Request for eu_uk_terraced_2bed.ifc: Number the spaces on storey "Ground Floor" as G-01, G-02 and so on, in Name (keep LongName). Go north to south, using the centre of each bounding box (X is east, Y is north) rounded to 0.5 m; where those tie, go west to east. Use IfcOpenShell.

First a look at what the model holds.

```python
import ifcopenshell
import ifcopenshell.util.element
import ifcopenshell.util.placement

model = ifcopenshell.open("eu_uk_terraced_2bed.ifc")
print(model.schema)
storey = next(s for s in model.by_type("IfcBuildingStorey") if s.Name == "Ground Floor")
spaces = [e for e in ifcopenshell.util.element.get_decomposition(storey) if e.is_a("IfcSpace")]
for e in sorted(spaces, key=lambda e: e.id()):
    origin = ifcopenshell.util.placement.get_local_placement(e.ObjectPlacement)[:3, 3]
    print(e.id(), e.Name, e.LongName, origin.round(2) + 0.0, sep=" | ")
```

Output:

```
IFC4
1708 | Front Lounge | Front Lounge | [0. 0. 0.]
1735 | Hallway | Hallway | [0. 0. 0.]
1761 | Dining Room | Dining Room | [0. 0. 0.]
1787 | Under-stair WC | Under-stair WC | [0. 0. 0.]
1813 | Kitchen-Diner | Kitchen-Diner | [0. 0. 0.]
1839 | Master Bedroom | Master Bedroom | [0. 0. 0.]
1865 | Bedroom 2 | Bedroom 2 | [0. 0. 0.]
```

```python
import ifcopenshell
import ifcopenshell.geom
import ifcopenshell.util.element
import ifcopenshell.util.shape

model = ifcopenshell.open("eu_uk_terraced_2bed.ifc")
settings = ifcopenshell.geom.settings()
settings.set("use-world-coords", True)


def centre(element):
    shape = ifcopenshell.geom.create_shape(settings, element)
    return ifcopenshell.util.shape.get_bbox_centroid(shape.geometry)


storey = next(s for s in model.by_type("IfcBuildingStorey") if s.Name == "Ground Floor")
spaces = [e for e in ifcopenshell.util.element.get_decomposition(storey) if e.is_a("IfcSpace")]

# Insertion points can sit at a corner or the storey origin, so sort by the geometry (in metres).
centres = {e: centre(e) for e in spaces}
spaces.sort(key=lambda e: (-round(centres[e][1] / 0.5), centres[e][0]))

for i, e in enumerate(spaces, start=1):
    number = f"G-{i:02d}"
    e.Name = number
    print(e.id(), number)

model.write("eu_uk_terraced_2bed_v2.ifc")
```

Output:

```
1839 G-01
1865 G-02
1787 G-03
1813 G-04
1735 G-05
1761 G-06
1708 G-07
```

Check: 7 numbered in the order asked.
